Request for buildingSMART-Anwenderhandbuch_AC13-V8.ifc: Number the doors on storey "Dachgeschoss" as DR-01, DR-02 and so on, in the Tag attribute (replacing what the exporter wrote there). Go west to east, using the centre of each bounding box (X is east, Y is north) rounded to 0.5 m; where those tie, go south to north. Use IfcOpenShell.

First a look at what the model holds.

```python
import ifcopenshell
import ifcopenshell.util.element
import ifcopenshell.util.placement

model = ifcopenshell.open("buildingSMART-Anwenderhandbuch_AC13-V8.ifc")
print(model.schema)
storey = next(s for s in model.by_type("IfcBuildingStorey") if s.Name == "Dachgeschoss")
doors = [e for e in ifcopenshell.util.element.get_decomposition(storey) if e.is_a("IfcDoor")]
for e in sorted(doors, key=lambda e: e.id()):
    origin = ifcopenshell.util.placement.get_local_placement(e.ObjectPlacement)[:3, 3]
    print(e.id(), e.Tag, e.Name, origin.round(2) + 0.0, sep=" | ")
```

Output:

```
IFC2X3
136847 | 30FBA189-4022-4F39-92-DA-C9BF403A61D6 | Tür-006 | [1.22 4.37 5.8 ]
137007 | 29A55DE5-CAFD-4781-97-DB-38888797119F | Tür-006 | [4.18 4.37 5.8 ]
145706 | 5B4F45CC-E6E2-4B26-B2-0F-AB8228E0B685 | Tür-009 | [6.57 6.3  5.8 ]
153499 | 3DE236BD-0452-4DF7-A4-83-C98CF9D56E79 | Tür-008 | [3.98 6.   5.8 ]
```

```python
import ifcopenshell
import ifcopenshell.geom
import ifcopenshell.util.element
import ifcopenshell.util.shape

model = ifcopenshell.open("buildingSMART-Anwenderhandbuch_AC13-V8.ifc")
settings = ifcopenshell.geom.settings()
settings.set("use-world-coords", True)


def centre(element):
    shape = ifcopenshell.geom.create_shape(settings, element)
    return ifcopenshell.util.shape.get_bbox_centroid(shape.geometry)


storey = next(s for s in model.by_type("IfcBuildingStorey") if s.Name == "Dachgeschoss")
doors = [e for e in ifcopenshell.util.element.get_decomposition(storey) if e.is_a("IfcDoor")]

# Insertion points can sit at a corner or the storey origin, so sort by the geometry (in metres).
centres = {e: centre(e) for e in doors}
doors.sort(key=lambda e: (round(centres[e][0] / 0.5), centres[e][1]))

for i, e in enumerate(doors, start=1):
    number = f"DR-{i:02d}"
    e.Tag = number
    print(e.id(), number)

model.write("buildingSMART-Anwenderhandbuch_AC13-V8-out.ifc")
```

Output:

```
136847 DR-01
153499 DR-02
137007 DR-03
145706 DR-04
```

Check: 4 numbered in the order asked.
